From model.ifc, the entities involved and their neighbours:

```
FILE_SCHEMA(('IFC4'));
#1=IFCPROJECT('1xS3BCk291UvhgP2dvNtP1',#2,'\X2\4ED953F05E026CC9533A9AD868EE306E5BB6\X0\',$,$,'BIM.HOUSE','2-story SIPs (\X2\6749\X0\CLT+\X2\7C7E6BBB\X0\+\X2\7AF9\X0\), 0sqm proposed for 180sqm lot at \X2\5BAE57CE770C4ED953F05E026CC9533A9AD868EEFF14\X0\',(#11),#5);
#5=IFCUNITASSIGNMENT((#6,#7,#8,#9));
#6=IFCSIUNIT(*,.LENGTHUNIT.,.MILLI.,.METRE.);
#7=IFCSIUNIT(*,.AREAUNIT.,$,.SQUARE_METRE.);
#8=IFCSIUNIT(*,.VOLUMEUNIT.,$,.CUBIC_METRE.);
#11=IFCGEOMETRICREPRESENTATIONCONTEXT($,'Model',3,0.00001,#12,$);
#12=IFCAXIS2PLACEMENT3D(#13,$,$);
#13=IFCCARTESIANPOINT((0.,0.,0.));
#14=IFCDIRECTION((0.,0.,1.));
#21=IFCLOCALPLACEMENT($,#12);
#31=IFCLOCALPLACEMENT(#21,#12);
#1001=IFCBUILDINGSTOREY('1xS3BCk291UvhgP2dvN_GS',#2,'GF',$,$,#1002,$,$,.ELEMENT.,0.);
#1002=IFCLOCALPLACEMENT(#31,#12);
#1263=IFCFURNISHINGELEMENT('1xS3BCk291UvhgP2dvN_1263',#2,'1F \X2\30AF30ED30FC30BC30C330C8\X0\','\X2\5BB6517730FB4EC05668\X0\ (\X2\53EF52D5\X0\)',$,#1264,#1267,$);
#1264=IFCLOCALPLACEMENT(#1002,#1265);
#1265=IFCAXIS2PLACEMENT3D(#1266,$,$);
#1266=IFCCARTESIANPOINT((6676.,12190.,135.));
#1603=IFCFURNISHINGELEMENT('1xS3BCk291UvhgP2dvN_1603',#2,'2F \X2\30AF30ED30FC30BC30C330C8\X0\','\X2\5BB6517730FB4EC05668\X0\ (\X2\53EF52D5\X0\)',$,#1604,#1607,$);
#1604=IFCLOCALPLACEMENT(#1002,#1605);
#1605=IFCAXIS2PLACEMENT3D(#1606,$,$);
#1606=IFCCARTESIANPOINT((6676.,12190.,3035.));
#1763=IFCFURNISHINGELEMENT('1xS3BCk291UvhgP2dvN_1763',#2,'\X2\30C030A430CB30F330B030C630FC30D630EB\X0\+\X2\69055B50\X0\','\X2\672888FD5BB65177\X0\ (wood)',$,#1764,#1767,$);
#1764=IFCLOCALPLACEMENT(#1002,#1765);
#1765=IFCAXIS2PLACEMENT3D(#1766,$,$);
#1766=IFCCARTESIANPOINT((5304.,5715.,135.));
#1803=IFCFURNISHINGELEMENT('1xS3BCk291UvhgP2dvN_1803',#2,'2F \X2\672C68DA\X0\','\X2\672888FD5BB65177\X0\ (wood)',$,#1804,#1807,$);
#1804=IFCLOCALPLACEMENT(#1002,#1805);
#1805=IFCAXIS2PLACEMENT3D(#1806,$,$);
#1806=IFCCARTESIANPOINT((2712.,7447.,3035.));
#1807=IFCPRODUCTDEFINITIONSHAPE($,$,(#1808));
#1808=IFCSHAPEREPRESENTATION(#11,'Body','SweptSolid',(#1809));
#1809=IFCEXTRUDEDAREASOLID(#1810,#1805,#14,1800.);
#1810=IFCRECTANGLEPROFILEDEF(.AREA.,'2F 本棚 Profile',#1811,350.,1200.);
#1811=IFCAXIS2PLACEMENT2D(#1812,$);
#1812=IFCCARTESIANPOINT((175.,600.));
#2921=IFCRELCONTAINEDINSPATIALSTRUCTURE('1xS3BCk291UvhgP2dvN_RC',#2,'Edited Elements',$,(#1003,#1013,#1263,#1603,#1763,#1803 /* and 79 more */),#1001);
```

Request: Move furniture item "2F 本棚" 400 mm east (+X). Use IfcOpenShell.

```python
import ifcopenshell
import ifcopenshell.api.geometry
import ifcopenshell.util.placement

model = ifcopenshell.open("model.ifc")

item = model.by_id(1803)
matrix = ifcopenshell.util.placement.get_local_placement(item.ObjectPlacement)
matrix[0, 3] += 400.0
ifcopenshell.api.geometry.edit_object_placement(model, product=item, matrix=matrix, is_si=False)

print(ifcopenshell.util.placement.get_local_placement(item.ObjectPlacement).round(3) + 0.0)

model.write("model_v2.ifc")
```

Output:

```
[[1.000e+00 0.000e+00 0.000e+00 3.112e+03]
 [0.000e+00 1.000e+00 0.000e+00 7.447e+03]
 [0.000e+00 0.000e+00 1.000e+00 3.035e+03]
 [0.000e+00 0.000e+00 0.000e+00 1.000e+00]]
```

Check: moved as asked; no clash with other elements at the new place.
